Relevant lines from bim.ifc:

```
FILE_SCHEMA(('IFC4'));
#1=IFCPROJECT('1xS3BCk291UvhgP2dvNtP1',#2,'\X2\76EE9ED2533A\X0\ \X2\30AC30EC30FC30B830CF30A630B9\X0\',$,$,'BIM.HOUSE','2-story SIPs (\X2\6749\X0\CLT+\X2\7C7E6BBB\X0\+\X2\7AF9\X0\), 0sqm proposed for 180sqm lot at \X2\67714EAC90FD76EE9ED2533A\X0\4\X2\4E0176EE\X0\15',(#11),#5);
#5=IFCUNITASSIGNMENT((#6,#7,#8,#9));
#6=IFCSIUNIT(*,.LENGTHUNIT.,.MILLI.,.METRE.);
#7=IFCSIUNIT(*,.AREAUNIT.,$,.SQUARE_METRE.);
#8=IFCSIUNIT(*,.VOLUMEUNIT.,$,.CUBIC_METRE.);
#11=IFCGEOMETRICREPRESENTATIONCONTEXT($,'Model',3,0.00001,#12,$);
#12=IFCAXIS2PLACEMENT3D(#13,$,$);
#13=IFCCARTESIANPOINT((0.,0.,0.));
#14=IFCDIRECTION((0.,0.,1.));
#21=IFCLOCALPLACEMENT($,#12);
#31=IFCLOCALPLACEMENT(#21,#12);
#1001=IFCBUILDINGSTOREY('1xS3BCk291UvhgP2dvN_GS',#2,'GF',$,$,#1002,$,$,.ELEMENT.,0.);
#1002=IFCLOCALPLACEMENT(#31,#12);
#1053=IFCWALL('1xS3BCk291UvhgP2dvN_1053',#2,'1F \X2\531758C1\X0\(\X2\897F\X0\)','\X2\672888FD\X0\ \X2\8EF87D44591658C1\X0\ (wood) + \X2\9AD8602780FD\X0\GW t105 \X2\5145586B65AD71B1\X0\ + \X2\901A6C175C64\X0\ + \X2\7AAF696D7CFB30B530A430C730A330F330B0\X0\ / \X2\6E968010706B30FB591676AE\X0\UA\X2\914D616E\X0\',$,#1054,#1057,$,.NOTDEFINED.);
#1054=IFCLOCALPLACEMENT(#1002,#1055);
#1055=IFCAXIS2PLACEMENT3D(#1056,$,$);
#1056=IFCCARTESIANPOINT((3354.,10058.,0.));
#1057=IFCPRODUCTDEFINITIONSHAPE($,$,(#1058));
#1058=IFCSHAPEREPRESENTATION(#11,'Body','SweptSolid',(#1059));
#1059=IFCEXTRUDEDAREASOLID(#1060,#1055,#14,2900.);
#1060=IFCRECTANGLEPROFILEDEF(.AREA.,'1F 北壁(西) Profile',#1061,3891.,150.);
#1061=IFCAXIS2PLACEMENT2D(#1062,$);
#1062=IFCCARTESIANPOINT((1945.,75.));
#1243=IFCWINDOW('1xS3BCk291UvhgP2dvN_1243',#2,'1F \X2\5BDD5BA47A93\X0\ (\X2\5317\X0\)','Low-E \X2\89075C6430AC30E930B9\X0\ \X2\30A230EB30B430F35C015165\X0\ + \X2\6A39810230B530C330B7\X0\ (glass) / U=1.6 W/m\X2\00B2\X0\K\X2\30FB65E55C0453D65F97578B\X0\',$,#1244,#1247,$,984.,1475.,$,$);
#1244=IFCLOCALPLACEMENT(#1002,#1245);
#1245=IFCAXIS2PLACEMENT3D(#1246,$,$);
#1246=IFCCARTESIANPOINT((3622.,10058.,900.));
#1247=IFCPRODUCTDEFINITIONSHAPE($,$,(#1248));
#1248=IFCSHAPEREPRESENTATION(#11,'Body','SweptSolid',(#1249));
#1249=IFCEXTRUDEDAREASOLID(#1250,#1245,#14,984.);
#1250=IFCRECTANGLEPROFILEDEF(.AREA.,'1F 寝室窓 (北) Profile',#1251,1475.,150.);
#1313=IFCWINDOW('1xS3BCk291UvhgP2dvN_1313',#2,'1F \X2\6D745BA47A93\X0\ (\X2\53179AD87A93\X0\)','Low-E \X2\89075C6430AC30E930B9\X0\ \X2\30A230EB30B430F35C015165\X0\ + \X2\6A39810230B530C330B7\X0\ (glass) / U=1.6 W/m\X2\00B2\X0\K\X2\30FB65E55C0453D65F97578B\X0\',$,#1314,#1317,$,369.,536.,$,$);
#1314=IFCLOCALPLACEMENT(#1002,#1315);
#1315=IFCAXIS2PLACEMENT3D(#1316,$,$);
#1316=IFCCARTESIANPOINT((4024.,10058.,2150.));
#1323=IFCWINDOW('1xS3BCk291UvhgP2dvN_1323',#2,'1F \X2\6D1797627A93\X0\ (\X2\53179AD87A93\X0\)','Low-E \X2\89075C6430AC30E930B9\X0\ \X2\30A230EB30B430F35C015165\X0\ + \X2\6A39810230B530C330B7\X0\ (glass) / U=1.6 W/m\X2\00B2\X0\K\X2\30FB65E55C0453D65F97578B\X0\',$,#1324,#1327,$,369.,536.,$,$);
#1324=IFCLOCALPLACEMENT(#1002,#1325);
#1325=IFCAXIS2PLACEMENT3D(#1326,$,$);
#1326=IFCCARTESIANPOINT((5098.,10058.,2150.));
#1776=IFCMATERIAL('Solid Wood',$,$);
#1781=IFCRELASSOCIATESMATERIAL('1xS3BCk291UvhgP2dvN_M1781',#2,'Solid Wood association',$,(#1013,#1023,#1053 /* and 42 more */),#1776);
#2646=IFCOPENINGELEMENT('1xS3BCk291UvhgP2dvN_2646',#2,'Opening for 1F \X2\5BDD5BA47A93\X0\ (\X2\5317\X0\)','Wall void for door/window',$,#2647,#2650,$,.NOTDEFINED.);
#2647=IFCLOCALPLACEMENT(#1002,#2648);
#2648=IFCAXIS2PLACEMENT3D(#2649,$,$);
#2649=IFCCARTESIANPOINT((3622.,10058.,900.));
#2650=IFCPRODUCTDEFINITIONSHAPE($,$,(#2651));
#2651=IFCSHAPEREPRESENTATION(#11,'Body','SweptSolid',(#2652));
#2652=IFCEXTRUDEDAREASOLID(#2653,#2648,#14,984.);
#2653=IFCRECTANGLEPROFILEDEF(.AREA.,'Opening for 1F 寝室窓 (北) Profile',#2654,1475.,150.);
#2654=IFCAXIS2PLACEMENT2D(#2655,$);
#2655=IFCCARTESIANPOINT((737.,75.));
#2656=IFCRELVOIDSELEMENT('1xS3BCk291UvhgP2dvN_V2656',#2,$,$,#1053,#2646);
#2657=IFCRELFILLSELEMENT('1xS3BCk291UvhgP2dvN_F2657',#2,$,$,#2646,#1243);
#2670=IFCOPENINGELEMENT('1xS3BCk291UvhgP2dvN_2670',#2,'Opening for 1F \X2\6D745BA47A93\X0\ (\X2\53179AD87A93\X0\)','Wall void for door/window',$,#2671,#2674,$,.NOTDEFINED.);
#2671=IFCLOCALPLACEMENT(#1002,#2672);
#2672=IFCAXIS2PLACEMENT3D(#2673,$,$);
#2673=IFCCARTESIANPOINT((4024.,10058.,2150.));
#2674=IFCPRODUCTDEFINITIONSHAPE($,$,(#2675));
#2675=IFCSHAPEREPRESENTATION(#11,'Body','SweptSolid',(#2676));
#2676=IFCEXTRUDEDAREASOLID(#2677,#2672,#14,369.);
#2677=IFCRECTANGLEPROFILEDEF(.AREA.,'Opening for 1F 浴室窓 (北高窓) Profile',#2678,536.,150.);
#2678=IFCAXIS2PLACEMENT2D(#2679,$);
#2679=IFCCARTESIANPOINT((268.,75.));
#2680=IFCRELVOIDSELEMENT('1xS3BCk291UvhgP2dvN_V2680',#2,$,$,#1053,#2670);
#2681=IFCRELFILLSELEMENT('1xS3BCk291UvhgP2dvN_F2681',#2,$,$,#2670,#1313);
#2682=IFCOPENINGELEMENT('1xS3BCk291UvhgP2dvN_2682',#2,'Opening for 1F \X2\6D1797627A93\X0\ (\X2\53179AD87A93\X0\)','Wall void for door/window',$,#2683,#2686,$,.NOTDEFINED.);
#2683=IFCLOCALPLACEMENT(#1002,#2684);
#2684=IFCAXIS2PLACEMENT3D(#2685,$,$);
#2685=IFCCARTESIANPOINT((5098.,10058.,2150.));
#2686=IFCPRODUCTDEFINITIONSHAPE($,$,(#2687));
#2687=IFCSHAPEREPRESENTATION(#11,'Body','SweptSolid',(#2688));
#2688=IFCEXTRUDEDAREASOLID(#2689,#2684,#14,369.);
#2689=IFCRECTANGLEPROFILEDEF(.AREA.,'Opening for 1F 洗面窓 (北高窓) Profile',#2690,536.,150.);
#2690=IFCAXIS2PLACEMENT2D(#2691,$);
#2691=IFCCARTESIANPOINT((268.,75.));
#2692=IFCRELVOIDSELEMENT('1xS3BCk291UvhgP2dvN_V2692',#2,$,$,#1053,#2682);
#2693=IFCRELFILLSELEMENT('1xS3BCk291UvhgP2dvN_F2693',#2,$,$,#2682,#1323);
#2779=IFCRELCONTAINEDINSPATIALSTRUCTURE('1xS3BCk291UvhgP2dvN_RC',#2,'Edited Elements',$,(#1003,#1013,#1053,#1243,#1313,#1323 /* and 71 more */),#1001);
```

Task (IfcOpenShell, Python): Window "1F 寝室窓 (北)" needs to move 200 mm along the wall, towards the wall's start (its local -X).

```python
import ifcopenshell
import ifcopenshell.api.geometry
import ifcopenshell.util.placement
import ifcopenshell.util.unit

model = ifcopenshell.open("bim.ifc")
unit_scale = ifcopenshell.util.unit.calculate_unit_scale(model)

window = model.by_guid("1xS3BCk291UvhgP2dvN_1243")
opening = window.FillsVoids[0].RelatingOpeningElement
wall = opening.VoidsElements[0].RelatingBuildingElement

wall_matrix = ifcopenshell.util.placement.get_local_placement(wall.ObjectPlacement)
shift = wall_matrix[:3, 0] * -0.2 / unit_scale
before = ifcopenshell.util.placement.get_local_placement(window.ObjectPlacement)[:3, 3].copy()

# The window is not placed relative to its opening, so move both.
for product in (opening, window):
    matrix = ifcopenshell.util.placement.get_local_placement(product.ObjectPlacement)
    matrix[:3, 3] += shift
    ifcopenshell.api.geometry.edit_object_placement(model, product=product, matrix=matrix, is_si=False)

after = ifcopenshell.util.placement.get_local_placement(window.ObjectPlacement)[:3, 3]
print("window moved by", (after - before).round(3) + 0.0)

model.write("bim_updated.ifc")
```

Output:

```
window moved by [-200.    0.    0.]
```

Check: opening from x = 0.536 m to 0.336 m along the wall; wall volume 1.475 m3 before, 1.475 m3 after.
